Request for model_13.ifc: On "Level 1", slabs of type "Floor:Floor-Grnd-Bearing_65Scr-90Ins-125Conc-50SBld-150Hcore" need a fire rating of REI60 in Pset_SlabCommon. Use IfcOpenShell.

First a look at what the model holds.

```python
import ifcopenshell
import ifcopenshell.util.element

model = ifcopenshell.open("model_13.ifc")
print(model.schema)
storey = next(s for s in model.by_type("IfcBuildingStorey") if s.Name == "Level 1")
slabs = [e for e in ifcopenshell.util.element.get_decomposition(storey) if e.is_a("IfcSlab")]
seen = {}
for e in slabs:
    element_type = ifcopenshell.util.element.get_type(e)
    key = (element_type.Name if element_type != e and element_type else None, ifcopenshell.util.element.get_pset(e, "Pset_SlabCommon", "FireRating"))
    seen[key] = seen.get(key, 0) + 1
for (name, value), count in sorted(seen.items(), key=str):
    print(count, "x", name, "|", value)
```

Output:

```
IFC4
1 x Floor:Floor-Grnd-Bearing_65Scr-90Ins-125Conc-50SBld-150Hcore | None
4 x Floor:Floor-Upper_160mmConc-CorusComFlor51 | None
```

```python
import ifcopenshell
import ifcopenshell.api.pset
import ifcopenshell.util.element

model = ifcopenshell.open("model_13.ifc")

storey = next(s for s in model.by_type("IfcBuildingStorey") if s.Name == "Level 1")
slabs = [e for e in ifcopenshell.util.element.get_decomposition(storey) if e.is_a("IfcSlab")]

count = 0
for e in slabs:
    element_type = ifcopenshell.util.element.get_type(e)
    if element_type in (None, e) or element_type.Name != "Floor:Floor-Grnd-Bearing_65Scr-90Ins-125Conc-50SBld-150Hcore":
        continue
    # add_pset returns the element's existing set when there is one.
    pset = ifcopenshell.api.pset.add_pset(model, product=e, name="Pset_SlabCommon")
    ifcopenshell.api.pset.edit_pset(model, pset=pset, properties={"FireRating": "REI60"})
    count += 1

print(count, "slabs updated")

model.write("model_13_edited.ifc")
```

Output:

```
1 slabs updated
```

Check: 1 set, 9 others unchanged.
